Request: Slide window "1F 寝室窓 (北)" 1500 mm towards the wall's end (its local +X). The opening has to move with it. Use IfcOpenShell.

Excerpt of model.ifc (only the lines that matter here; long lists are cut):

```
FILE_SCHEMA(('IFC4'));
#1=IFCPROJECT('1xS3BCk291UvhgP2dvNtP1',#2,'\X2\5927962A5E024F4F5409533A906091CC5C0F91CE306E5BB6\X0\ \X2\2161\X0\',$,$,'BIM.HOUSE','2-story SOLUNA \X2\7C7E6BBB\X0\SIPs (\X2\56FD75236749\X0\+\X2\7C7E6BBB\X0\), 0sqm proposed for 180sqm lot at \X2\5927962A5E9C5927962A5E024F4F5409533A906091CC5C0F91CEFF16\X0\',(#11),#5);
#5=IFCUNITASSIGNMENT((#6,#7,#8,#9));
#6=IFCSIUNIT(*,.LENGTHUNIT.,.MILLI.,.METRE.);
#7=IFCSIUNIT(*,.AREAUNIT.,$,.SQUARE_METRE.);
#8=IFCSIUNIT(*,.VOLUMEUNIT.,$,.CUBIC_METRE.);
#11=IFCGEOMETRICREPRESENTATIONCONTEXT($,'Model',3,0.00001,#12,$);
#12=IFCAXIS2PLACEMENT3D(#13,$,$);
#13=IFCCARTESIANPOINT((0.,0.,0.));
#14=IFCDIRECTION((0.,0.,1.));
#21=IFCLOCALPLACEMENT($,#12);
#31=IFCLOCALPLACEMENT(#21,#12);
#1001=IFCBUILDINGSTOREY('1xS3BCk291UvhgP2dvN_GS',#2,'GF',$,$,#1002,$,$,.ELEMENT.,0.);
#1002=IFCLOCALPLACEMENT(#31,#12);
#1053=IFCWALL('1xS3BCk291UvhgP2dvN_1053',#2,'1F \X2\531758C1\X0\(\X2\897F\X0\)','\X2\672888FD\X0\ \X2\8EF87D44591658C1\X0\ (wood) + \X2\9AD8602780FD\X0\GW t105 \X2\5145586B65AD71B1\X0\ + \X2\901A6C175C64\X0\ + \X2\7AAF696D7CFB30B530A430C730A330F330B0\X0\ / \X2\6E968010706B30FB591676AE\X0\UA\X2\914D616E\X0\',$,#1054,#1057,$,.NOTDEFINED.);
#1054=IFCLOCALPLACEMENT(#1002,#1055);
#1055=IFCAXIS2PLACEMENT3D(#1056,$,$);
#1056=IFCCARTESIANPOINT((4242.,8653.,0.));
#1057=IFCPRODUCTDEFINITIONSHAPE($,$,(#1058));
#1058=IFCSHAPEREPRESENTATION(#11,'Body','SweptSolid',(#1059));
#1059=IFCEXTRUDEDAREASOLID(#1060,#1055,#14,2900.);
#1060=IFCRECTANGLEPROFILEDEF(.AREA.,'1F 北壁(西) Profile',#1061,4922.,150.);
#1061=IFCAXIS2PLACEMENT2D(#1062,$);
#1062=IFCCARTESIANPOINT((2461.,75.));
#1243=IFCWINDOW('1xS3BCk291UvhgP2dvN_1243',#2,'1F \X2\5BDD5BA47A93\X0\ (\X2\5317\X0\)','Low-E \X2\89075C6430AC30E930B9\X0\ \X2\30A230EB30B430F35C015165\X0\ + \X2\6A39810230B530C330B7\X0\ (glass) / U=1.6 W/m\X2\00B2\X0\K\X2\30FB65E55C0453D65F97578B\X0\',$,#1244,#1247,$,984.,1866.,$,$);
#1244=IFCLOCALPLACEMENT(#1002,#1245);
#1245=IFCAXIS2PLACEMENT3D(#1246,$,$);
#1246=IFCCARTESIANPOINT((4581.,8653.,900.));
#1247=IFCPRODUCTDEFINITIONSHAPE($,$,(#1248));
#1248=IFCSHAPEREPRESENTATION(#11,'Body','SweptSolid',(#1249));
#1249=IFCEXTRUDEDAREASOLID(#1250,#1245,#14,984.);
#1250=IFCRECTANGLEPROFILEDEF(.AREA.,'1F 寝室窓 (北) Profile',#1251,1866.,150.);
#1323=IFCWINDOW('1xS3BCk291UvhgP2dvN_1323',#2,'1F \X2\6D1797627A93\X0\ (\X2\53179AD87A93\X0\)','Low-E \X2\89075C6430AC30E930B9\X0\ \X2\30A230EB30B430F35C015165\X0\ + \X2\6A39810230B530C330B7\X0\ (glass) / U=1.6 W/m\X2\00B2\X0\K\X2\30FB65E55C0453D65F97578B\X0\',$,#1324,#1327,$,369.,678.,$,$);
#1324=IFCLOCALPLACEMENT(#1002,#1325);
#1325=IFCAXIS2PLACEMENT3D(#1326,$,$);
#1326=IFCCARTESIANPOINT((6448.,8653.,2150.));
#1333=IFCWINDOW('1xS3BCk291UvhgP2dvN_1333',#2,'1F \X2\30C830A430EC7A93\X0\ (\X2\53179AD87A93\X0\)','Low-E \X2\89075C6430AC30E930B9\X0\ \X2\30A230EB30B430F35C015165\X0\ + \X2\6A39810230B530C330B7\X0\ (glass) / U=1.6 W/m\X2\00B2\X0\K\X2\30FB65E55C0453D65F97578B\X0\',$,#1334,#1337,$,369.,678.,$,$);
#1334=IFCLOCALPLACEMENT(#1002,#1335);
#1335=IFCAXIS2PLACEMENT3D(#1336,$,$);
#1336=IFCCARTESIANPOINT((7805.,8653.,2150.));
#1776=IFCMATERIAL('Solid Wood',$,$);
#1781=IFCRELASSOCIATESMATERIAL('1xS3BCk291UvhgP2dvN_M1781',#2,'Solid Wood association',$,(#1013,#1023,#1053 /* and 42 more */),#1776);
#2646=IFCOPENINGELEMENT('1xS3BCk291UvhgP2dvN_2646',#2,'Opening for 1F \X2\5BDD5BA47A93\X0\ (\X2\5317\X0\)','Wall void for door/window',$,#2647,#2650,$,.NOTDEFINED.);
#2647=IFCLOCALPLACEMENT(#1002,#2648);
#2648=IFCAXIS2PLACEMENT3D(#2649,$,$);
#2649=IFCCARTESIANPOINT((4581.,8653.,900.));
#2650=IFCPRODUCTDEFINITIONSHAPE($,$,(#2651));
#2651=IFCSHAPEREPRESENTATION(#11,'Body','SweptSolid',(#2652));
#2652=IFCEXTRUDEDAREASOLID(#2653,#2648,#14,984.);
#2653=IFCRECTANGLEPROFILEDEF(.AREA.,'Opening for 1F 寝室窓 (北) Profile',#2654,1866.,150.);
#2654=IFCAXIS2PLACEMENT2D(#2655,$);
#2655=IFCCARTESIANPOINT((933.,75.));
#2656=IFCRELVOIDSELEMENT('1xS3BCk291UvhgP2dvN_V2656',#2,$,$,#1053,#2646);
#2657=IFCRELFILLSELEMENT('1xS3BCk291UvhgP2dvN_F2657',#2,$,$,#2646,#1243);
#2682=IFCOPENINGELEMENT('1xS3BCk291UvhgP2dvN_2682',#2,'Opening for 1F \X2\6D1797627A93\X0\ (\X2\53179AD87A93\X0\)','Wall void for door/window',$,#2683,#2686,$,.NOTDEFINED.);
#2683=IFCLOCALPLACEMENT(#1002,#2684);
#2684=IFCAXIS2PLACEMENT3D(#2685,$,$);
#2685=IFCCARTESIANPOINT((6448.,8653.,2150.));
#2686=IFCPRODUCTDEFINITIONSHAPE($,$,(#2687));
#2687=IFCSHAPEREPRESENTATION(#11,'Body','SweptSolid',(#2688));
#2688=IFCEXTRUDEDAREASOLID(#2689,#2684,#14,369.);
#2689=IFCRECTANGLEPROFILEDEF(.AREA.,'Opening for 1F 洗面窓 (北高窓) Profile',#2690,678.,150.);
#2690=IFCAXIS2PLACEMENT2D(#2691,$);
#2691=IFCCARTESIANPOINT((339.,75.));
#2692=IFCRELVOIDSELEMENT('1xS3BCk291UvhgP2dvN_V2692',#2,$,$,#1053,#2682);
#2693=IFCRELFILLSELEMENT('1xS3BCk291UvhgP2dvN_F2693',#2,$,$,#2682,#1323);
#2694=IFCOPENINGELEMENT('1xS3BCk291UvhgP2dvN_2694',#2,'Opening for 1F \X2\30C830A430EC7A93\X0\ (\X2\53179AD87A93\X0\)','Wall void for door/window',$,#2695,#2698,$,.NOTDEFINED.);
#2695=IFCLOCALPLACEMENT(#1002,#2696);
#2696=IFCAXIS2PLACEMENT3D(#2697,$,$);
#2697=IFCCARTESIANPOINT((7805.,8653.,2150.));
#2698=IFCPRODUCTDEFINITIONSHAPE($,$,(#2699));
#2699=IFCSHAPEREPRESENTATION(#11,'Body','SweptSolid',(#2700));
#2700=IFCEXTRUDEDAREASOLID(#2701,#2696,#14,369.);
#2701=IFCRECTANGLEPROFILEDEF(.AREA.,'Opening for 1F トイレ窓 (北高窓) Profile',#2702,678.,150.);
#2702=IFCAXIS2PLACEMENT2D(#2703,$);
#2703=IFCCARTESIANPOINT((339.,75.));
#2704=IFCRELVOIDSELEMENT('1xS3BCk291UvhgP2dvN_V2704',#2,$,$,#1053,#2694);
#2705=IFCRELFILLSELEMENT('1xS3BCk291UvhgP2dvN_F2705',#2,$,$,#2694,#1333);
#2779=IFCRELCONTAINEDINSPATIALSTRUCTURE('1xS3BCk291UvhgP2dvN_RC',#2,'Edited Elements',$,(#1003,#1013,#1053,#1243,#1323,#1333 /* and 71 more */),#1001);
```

```python
import ifcopenshell
import ifcopenshell.api.geometry
import ifcopenshell.util.placement
import ifcopenshell.util.unit

model = ifcopenshell.open("model.ifc")
unit_scale = ifcopenshell.util.unit.calculate_unit_scale(model)

window = model.by_id(1243)
opening = window.FillsVoids[0].RelatingOpeningElement
wall = opening.VoidsElements[0].RelatingBuildingElement

wall_matrix = ifcopenshell.util.placement.get_local_placement(wall.ObjectPlacement)
shift = wall_matrix[:3, 0] * 1.5 / unit_scale
before = ifcopenshell.util.placement.get_local_placement(window.ObjectPlacement)[:3, 3].copy()

# The window is not placed relative to its opening, so move both.
for product in (opening, window):
    matrix = ifcopenshell.util.placement.get_local_placement(product.ObjectPlacement)
    matrix[:3, 3] += shift
    ifcopenshell.api.geometry.edit_object_placement(model, product=product, matrix=matrix, is_si=False)

after = ifcopenshell.util.placement.get_local_placement(window.ObjectPlacement)[:3, 3]
print("window moved by", (after - before).round(3) + 0.0)

model.write("model-out.ifc")
```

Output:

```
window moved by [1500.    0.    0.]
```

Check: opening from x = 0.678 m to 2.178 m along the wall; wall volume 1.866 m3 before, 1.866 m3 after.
